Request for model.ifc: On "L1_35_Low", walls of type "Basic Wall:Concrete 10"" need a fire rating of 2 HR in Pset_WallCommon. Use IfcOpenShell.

First a look at what the model holds.

```python
import ifcopenshell
import ifcopenshell.util.element

model = ifcopenshell.open("model.ifc")
print(model.schema)
storey = next(s for s in model.by_type("IfcBuildingStorey") if s.Name == "L1_35_Low")
walls = [e for e in ifcopenshell.util.element.get_decomposition(storey) if e.is_a("IfcWall")]
seen = {}
for e in walls:
    element_type = ifcopenshell.util.element.get_type(e)
    key = (element_type.Name if element_type != e and element_type else None, ifcopenshell.util.element.get_pset(e, "Pset_WallCommon", "FireRating"))
    seen[key] = seen.get(key, 0) + 1
for (name, value), count in sorted(seen.items(), key=str):
    print(count, "x", name, "|", value)
```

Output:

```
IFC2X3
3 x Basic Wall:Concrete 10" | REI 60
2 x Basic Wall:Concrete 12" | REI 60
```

```python
import ifcopenshell
import ifcopenshell.api.pset
import ifcopenshell.util.element

model = ifcopenshell.open("model.ifc")

storey = next(s for s in model.by_type("IfcBuildingStorey") if s.Name == "L1_35_Low")
walls = [e for e in ifcopenshell.util.element.get_decomposition(storey) if e.is_a("IfcWall")]

count = 0
for e in walls:
    element_type = ifcopenshell.util.element.get_type(e)
    if element_type in (None, e) or element_type.Name != 'Basic Wall:Concrete 10"':
        continue
    # add_pset returns the element's existing set when there is one.
    pset = ifcopenshell.api.pset.add_pset(model, product=e, name="Pset_WallCommon")
    ifcopenshell.api.pset.edit_pset(model, pset=pset, properties={"FireRating": "2 HR"})
    count += 1

print(count, "walls updated")

model.write("model_v2.ifc")
```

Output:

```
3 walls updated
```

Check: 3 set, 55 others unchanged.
